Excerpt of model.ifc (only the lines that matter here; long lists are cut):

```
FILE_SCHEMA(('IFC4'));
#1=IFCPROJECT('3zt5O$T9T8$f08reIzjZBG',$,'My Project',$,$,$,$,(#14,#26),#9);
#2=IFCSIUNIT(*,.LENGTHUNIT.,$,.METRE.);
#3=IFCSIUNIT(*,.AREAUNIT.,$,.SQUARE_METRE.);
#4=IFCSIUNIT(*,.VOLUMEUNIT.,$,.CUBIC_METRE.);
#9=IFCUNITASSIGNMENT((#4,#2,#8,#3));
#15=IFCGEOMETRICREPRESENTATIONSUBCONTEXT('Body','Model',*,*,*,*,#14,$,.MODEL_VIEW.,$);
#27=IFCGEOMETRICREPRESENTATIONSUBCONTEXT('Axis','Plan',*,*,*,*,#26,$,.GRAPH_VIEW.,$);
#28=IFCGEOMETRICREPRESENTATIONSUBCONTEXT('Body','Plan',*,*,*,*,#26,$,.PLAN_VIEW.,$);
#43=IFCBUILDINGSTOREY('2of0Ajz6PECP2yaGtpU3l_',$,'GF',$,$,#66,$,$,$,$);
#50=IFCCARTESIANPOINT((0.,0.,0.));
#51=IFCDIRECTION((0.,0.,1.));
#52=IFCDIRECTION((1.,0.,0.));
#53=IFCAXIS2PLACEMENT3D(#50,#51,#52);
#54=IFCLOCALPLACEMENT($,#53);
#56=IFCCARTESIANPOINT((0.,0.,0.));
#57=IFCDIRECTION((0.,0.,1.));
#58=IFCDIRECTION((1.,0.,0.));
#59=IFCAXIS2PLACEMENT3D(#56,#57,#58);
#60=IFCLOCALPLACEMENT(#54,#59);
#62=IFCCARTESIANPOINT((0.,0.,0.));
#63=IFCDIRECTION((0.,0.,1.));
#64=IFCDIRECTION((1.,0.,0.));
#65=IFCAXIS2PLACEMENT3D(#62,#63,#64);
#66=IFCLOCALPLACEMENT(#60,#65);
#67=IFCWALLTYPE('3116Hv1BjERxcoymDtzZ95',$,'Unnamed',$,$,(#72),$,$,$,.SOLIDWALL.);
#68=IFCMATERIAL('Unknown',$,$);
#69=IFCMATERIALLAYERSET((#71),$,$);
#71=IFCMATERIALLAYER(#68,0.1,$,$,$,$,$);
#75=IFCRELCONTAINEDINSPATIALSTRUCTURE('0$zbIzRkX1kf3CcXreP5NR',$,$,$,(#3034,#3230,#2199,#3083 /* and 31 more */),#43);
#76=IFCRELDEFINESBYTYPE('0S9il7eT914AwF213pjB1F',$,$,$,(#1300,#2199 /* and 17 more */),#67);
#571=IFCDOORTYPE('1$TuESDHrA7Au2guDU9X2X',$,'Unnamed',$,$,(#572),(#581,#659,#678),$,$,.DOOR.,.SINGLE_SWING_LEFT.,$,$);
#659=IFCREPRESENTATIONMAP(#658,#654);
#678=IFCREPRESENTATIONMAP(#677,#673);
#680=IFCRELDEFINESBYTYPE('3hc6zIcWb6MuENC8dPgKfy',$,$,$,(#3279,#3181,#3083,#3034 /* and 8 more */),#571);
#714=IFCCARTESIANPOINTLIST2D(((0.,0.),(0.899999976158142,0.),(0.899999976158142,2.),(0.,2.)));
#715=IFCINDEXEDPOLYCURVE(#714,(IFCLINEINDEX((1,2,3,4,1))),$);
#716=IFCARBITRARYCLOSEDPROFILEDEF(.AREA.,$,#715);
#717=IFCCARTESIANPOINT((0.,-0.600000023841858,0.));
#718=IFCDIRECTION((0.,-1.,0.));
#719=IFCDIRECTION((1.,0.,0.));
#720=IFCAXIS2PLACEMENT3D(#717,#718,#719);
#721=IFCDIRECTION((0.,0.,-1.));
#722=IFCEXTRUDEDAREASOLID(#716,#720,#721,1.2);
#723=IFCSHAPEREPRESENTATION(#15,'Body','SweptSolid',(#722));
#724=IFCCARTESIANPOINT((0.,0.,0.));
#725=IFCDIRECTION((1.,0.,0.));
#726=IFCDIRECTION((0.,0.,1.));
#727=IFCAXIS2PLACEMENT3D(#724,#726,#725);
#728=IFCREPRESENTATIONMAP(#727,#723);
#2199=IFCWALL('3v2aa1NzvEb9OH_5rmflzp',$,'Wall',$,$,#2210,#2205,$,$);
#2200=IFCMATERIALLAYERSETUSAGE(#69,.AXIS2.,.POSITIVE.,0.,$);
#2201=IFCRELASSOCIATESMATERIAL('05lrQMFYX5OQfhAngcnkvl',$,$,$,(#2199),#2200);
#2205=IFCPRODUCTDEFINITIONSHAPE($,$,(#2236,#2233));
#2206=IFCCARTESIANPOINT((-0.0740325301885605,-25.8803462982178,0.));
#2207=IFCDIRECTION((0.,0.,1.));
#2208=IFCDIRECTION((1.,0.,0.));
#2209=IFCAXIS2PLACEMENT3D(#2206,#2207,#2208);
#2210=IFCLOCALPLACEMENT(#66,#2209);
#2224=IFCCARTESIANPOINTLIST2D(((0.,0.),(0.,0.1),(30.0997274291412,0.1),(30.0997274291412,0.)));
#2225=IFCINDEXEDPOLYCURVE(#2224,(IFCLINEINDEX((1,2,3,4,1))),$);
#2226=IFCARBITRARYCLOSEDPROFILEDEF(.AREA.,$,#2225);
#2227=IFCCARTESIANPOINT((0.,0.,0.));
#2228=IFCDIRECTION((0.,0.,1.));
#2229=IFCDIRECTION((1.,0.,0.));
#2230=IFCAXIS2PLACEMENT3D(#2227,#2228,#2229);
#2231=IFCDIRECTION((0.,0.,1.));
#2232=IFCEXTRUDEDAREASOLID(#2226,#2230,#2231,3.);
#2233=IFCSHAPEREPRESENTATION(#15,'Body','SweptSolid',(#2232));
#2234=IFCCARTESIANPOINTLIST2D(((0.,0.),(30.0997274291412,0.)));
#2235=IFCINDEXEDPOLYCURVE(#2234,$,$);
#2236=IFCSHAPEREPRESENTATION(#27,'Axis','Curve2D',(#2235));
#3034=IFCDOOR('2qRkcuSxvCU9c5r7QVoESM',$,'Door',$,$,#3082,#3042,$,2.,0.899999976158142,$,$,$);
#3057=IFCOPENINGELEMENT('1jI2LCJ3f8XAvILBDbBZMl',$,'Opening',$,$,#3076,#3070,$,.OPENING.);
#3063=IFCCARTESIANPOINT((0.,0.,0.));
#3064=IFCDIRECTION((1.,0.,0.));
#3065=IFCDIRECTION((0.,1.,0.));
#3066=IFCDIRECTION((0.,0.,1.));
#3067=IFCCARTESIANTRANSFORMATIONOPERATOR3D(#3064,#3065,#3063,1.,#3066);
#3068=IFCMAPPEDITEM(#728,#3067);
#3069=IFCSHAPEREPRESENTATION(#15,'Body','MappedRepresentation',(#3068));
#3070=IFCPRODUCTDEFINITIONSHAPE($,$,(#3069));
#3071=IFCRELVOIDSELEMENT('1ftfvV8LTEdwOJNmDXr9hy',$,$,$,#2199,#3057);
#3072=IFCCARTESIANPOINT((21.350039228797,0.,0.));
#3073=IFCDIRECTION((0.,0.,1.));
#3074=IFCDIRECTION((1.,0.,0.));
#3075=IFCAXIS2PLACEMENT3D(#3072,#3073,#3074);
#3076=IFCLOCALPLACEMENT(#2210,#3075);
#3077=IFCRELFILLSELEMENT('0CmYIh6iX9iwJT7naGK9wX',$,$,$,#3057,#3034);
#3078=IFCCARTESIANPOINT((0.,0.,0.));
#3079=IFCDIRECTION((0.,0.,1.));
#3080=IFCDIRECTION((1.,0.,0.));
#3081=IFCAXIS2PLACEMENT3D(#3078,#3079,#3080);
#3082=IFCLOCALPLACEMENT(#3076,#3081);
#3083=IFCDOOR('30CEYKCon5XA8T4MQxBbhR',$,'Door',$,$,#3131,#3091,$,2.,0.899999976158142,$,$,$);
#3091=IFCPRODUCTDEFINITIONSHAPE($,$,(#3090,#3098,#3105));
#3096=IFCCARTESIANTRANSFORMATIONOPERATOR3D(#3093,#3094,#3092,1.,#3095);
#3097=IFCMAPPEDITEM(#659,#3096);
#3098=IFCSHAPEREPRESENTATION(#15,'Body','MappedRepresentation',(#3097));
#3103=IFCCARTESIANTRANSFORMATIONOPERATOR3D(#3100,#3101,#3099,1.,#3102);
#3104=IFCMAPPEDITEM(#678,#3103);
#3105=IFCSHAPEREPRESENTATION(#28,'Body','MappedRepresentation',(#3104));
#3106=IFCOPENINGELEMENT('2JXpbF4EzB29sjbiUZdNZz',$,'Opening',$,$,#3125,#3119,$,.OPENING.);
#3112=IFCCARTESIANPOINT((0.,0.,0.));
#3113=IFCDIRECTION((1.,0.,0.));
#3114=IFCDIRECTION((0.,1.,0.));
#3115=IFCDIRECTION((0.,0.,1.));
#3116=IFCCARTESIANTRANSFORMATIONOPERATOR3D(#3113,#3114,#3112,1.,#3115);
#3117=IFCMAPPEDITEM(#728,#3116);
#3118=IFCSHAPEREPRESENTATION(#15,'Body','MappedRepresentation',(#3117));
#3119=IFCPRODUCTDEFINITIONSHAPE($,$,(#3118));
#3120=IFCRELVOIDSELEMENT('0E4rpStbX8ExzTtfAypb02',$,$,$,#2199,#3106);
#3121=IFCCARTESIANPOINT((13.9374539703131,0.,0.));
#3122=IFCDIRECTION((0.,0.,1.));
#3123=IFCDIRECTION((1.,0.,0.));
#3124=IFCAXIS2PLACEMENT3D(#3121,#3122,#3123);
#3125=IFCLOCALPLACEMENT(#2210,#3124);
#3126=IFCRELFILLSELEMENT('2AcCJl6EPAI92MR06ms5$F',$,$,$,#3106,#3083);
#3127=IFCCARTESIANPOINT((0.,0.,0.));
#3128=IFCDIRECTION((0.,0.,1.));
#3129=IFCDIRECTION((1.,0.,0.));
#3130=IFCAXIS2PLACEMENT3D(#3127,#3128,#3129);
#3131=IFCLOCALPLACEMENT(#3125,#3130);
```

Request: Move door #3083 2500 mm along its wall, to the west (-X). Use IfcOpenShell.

```python
import ifcopenshell
import ifcopenshell.api.geometry
import ifcopenshell.util.placement
import ifcopenshell.util.unit

model = ifcopenshell.open("model.ifc")
unit_scale = ifcopenshell.util.unit.calculate_unit_scale(model)

door = model.by_id(3083)
opening = door.FillsVoids[0].RelatingOpeningElement
wall = opening.VoidsElements[0].RelatingBuildingElement

wall_matrix = ifcopenshell.util.placement.get_local_placement(wall.ObjectPlacement)
shift = wall_matrix[:3, 0] * -2.5 / unit_scale
before = ifcopenshell.util.placement.get_local_placement(door.ObjectPlacement)[:3, 3].copy()

# The door is placed relative to its opening, so it follows when the opening moves.
matrix = ifcopenshell.util.placement.get_local_placement(opening.ObjectPlacement)
matrix[:3, 3] += shift
ifcopenshell.api.geometry.edit_object_placement(
    model, product=opening, matrix=matrix, is_si=False, should_transform_children=True
)

after = ifcopenshell.util.placement.get_local_placement(door.ObjectPlacement)[:3, 3]
print("door moved by", (after - before).round(3) + 0.0)

model.write("model_rev.ifc")
```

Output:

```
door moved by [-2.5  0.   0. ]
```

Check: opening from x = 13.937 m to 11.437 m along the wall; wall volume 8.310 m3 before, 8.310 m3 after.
